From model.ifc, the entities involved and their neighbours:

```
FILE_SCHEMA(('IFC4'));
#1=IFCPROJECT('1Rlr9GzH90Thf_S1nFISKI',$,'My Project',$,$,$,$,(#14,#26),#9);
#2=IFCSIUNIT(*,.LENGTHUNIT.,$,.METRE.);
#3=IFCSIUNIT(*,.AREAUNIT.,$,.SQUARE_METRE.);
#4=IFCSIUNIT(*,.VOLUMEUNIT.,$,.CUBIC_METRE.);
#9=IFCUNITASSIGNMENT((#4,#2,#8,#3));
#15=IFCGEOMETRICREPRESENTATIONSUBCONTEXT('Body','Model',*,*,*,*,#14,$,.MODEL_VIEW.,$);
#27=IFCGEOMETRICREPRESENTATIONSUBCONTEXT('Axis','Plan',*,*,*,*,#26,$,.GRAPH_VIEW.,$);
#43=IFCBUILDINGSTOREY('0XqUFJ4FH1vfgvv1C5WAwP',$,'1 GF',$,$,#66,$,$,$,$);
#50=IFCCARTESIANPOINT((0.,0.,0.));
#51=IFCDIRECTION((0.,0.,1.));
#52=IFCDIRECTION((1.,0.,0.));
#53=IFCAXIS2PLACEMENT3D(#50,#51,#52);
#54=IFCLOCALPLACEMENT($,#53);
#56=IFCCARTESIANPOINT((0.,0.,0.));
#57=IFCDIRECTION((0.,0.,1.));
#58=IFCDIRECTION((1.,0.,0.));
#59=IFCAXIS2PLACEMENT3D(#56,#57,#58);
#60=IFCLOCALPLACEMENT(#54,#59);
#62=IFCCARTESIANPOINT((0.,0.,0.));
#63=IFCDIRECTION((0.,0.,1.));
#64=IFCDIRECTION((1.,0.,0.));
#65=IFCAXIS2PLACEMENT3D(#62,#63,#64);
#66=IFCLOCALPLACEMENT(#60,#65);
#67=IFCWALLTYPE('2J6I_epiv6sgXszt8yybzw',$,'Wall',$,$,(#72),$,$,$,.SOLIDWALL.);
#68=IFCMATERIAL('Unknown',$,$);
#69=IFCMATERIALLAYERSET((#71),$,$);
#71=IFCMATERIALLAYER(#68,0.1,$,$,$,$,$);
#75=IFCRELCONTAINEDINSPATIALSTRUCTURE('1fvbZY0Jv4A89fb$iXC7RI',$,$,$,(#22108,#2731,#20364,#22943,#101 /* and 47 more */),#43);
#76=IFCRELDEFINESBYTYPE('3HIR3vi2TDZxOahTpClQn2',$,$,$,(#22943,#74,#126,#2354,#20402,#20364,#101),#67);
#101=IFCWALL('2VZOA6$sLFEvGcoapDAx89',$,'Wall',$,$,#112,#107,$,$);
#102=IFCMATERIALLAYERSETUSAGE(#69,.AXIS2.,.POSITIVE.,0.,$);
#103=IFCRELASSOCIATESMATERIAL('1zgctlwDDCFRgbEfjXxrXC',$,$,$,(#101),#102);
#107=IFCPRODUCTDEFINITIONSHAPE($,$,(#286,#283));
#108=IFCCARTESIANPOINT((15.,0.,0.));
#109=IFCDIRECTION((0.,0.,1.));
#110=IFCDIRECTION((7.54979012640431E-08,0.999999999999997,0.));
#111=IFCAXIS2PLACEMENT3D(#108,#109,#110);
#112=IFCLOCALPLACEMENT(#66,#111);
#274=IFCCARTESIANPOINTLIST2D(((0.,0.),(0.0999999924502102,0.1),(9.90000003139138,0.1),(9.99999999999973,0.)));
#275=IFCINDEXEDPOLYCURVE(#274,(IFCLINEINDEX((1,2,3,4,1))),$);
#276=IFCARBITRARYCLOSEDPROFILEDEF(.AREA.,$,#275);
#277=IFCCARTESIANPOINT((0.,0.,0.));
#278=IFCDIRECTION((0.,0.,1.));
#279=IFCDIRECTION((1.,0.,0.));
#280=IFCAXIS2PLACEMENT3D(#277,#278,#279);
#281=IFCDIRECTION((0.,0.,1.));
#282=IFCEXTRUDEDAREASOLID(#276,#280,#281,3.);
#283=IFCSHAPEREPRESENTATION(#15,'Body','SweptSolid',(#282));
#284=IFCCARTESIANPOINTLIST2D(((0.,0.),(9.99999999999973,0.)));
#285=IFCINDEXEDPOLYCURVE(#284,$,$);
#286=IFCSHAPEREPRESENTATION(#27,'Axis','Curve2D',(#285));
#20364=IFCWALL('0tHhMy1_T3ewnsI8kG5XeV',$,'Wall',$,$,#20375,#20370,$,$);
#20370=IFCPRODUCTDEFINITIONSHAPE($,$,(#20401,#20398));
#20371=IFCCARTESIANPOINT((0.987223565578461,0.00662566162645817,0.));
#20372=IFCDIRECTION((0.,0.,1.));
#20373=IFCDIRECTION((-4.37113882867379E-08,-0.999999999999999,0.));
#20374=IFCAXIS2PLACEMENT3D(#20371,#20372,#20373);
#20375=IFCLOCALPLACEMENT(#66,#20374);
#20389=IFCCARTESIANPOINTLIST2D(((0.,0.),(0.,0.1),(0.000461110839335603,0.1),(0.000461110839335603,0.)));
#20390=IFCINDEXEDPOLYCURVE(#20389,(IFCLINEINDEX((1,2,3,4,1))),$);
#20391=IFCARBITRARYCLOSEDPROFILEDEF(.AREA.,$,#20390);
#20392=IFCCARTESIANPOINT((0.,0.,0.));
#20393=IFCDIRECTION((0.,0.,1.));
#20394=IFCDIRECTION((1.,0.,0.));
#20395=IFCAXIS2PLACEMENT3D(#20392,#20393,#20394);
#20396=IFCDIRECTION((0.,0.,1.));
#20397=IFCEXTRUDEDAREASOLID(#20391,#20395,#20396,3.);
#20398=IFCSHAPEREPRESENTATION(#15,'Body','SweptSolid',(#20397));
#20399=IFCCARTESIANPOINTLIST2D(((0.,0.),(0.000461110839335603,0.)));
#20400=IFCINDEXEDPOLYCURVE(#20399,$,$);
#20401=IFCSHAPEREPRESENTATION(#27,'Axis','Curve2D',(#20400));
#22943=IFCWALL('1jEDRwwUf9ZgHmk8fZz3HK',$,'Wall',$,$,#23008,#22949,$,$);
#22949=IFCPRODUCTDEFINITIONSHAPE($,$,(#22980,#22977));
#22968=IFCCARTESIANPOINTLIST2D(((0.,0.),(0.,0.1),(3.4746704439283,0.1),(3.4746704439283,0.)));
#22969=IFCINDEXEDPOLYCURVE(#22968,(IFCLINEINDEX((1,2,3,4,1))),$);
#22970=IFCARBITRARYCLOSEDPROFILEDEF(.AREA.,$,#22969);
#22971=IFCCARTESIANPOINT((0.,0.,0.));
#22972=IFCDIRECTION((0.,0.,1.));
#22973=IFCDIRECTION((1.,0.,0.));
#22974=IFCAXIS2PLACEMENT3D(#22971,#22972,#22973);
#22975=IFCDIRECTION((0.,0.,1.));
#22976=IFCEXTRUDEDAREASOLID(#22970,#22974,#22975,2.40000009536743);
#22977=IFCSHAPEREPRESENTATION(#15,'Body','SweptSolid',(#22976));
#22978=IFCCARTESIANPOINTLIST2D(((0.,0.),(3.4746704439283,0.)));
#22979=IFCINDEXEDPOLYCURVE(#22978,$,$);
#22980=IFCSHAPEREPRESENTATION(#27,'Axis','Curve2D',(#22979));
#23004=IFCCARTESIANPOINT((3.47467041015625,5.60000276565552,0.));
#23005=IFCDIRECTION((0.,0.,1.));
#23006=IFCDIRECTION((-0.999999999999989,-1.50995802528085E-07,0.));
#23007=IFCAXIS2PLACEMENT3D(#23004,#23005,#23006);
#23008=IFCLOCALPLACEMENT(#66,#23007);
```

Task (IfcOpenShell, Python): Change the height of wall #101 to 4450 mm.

```python
import ifcopenshell
import ifcopenshell.geom
import ifcopenshell.util.representation
import ifcopenshell.util.shape
import ifcopenshell.util.unit

model = ifcopenshell.open("model.ifc")
unit_scale = ifcopenshell.util.unit.calculate_unit_scale(model)
settings = ifcopenshell.geom.settings()


def volume(element):
    """Net volume in cubic metres, openings subtracted."""
    shape = ifcopenshell.geom.create_shape(settings, element)
    return ifcopenshell.util.shape.get_volume(shape.geometry)


wall = model.by_guid("2VZOA6$sLFEvGcoapDAx89")
before = volume(wall)

body = ifcopenshell.util.representation.get_representation(wall, "Model", "Body")
solid = body.Items[0]
old_height = solid.Depth
solid.Depth = 4.45 / unit_scale
after = volume(wall)

print(f"height {old_height:g} -> {solid.Depth:g}, volume {before:.3f} -> {after:.3f} m3")

model.write("model-out.ifc")
```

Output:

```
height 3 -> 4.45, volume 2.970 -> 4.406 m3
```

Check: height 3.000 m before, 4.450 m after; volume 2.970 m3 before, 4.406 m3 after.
